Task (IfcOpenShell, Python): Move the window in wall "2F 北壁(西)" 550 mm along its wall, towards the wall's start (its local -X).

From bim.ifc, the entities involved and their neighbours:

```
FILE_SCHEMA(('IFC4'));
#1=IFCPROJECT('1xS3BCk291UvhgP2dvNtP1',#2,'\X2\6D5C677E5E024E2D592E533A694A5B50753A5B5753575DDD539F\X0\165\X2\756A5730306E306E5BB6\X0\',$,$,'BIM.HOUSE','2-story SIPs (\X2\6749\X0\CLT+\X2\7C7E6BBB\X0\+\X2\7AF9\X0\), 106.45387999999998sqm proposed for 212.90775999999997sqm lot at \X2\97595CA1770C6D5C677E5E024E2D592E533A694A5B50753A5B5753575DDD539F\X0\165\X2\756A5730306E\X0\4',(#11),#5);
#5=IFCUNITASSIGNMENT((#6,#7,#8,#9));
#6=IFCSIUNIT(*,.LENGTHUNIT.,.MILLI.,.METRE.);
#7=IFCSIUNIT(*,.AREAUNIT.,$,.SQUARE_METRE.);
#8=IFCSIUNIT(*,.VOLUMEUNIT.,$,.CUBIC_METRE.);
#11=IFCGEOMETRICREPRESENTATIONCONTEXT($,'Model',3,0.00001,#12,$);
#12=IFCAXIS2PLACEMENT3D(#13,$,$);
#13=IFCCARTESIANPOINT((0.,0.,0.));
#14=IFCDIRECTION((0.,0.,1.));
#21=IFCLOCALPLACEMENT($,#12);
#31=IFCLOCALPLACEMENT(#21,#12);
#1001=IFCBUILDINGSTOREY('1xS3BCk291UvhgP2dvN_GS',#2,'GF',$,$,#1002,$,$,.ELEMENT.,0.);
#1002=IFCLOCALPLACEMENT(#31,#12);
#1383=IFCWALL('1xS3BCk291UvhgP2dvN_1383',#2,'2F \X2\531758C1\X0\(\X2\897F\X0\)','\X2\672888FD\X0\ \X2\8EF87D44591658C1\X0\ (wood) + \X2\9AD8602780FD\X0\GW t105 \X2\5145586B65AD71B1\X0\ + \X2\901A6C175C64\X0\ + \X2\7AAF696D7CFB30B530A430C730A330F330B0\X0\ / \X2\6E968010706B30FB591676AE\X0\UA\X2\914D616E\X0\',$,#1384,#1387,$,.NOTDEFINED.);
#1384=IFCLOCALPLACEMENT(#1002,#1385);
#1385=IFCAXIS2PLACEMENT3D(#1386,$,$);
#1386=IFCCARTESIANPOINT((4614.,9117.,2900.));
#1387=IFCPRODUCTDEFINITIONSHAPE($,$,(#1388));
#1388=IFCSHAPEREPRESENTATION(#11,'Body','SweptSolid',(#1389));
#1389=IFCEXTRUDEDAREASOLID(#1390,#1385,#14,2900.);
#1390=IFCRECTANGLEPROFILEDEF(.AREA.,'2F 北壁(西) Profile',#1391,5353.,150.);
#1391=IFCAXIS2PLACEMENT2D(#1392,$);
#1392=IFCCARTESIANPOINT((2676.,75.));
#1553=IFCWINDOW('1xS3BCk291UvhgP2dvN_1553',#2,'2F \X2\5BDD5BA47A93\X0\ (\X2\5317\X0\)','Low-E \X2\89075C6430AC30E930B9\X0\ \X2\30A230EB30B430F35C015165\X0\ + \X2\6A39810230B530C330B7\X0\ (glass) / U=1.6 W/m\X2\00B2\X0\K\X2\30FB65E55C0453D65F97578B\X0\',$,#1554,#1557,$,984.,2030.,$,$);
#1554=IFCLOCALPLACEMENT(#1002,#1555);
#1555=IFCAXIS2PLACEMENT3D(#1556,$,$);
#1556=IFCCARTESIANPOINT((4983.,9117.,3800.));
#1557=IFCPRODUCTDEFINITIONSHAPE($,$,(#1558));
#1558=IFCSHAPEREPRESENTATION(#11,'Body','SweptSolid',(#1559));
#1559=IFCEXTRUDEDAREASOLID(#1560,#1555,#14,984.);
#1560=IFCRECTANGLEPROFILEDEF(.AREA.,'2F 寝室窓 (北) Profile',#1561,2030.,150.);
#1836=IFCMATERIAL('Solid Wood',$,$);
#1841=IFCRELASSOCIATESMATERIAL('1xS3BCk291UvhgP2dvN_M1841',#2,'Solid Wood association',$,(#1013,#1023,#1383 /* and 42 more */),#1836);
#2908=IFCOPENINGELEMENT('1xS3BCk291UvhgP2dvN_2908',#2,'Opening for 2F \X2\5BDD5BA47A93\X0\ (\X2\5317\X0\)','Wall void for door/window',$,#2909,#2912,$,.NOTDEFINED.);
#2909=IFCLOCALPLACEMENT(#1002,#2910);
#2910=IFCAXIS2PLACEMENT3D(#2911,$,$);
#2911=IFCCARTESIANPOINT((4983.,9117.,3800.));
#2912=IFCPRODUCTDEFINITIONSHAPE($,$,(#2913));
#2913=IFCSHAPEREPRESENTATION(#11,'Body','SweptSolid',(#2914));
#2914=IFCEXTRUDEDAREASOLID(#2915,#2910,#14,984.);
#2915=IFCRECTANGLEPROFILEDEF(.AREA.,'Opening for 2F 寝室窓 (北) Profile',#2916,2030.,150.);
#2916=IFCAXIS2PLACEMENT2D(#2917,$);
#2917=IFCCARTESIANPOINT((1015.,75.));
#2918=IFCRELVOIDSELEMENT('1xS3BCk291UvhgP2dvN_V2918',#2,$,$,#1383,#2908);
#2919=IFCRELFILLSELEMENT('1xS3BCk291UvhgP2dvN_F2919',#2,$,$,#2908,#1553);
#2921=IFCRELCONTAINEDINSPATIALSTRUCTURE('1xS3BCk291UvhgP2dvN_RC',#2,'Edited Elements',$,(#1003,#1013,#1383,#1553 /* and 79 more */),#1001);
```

```python
import ifcopenshell
import ifcopenshell.api.geometry
import ifcopenshell.util.placement
import ifcopenshell.util.unit

model = ifcopenshell.open("bim.ifc")
unit_scale = ifcopenshell.util.unit.calculate_unit_scale(model)

window = model.by_id(1553)
opening = window.FillsVoids[0].RelatingOpeningElement
wall = opening.VoidsElements[0].RelatingBuildingElement

wall_matrix = ifcopenshell.util.placement.get_local_placement(wall.ObjectPlacement)
shift = wall_matrix[:3, 0] * -0.55 / unit_scale
before = ifcopenshell.util.placement.get_local_placement(window.ObjectPlacement)[:3, 3].copy()

# The window is not placed relative to its opening, so move both.
for product in (opening, window):
    matrix = ifcopenshell.util.placement.get_local_placement(product.ObjectPlacement)
    matrix[:3, 3] += shift
    ifcopenshell.api.geometry.edit_object_placement(model, product=product, matrix=matrix, is_si=False)

after = ifcopenshell.util.placement.get_local_placement(window.ObjectPlacement)[:3, 3]
print("window moved by", (after - before).round(3) + 0.0)

model.write("bim_edited.ifc")
```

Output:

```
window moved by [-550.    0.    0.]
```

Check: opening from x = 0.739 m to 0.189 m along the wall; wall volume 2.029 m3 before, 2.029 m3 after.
